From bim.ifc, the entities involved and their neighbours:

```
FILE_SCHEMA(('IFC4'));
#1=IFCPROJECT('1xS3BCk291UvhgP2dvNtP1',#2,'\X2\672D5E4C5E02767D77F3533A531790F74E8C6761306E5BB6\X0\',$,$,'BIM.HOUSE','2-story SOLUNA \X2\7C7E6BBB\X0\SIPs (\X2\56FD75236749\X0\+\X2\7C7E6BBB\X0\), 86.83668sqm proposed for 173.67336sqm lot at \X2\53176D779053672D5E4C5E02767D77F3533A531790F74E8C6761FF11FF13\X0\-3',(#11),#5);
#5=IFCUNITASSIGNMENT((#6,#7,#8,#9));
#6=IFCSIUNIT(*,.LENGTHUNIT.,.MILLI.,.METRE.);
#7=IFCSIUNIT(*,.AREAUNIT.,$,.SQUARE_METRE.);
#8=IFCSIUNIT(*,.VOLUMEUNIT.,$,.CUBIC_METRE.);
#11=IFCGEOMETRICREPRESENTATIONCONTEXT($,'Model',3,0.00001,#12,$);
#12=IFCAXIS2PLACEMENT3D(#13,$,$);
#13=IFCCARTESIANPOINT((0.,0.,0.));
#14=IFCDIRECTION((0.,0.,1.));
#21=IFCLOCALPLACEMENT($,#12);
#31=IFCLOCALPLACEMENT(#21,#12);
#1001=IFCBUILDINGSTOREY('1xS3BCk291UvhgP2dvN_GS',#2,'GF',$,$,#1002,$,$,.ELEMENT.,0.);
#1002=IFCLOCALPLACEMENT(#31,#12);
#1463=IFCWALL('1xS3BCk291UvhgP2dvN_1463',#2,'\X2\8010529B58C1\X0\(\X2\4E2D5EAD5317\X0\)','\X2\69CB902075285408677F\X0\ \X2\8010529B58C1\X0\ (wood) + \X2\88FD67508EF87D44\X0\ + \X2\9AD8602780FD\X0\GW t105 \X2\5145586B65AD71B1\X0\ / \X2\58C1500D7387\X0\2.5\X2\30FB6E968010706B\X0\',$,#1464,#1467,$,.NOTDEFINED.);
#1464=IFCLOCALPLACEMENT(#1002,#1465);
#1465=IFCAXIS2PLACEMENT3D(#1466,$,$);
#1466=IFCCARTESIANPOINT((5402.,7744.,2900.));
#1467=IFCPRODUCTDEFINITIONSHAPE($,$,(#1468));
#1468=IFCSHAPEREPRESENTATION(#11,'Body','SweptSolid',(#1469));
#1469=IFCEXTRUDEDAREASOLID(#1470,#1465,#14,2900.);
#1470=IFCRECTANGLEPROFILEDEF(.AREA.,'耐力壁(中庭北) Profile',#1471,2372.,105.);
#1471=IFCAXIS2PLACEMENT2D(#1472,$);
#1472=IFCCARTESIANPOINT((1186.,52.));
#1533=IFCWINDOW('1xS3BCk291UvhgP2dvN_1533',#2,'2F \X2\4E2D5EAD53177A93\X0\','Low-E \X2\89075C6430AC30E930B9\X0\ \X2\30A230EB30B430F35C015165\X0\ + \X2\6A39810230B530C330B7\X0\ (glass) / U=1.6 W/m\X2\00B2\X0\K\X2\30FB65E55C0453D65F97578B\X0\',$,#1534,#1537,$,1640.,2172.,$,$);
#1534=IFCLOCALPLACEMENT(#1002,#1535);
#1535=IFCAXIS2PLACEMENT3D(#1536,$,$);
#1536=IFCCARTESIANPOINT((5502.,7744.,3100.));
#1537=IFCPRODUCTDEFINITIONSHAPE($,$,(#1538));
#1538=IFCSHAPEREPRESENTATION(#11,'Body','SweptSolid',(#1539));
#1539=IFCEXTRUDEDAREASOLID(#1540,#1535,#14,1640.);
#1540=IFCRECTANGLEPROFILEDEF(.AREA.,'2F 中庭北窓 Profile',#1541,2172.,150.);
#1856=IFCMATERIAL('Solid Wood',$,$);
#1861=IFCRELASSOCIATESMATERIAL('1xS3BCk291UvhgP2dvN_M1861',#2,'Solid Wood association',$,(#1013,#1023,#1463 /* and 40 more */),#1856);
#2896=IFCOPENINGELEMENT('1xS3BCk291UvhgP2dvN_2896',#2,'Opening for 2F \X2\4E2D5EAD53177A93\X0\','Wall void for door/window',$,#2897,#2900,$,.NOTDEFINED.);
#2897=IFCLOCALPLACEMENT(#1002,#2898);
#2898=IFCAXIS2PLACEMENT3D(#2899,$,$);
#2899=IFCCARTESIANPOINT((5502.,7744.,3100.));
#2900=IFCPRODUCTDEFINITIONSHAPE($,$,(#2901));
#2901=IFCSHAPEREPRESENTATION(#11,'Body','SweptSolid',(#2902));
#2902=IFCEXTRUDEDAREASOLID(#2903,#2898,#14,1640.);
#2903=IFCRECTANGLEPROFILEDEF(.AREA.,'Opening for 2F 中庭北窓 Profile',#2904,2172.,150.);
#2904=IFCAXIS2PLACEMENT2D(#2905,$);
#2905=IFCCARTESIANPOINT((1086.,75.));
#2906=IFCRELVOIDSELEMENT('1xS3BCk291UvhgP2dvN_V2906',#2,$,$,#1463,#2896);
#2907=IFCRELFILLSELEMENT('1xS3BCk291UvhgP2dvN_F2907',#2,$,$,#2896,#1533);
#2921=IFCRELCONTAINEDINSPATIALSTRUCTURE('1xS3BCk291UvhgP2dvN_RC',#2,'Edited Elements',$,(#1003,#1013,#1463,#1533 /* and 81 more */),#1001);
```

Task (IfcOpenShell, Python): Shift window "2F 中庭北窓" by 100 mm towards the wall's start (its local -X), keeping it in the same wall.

```python
import ifcopenshell
import ifcopenshell.api.geometry
import ifcopenshell.util.placement
import ifcopenshell.util.unit

model = ifcopenshell.open("bim.ifc")
unit_scale = ifcopenshell.util.unit.calculate_unit_scale(model)

window = model.by_guid("1xS3BCk291UvhgP2dvN_1533")
opening = window.FillsVoids[0].RelatingOpeningElement
wall = opening.VoidsElements[0].RelatingBuildingElement

wall_matrix = ifcopenshell.util.placement.get_local_placement(wall.ObjectPlacement)
shift = wall_matrix[:3, 0] * -0.1 / unit_scale
before = ifcopenshell.util.placement.get_local_placement(window.ObjectPlacement)[:3, 3].copy()

# The window is not placed relative to its opening, so move both.
for product in (opening, window):
    matrix = ifcopenshell.util.placement.get_local_placement(product.ObjectPlacement)
    matrix[:3, 3] += shift
    ifcopenshell.api.geometry.edit_object_placement(model, product=product, matrix=matrix, is_si=False)

after = ifcopenshell.util.placement.get_local_placement(window.ObjectPlacement)[:3, 3]
print("window moved by", (after - before).round(3) + 0.0)

model.write("bim_rev.ifc")
```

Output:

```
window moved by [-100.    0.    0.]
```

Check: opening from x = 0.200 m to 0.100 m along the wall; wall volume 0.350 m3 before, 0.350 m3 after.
